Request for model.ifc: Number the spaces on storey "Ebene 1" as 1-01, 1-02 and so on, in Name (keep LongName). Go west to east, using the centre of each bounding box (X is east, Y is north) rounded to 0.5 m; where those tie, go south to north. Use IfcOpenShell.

First a look at what the model holds.

```python
import ifcopenshell
import ifcopenshell.util.element
import ifcopenshell.util.placement

model = ifcopenshell.open("model.ifc")
print(model.schema)
storey = next(s for s in model.by_type("IfcBuildingStorey") if s.Name == "Ebene 1")
spaces = [e for e in ifcopenshell.util.element.get_decomposition(storey) if e.is_a("IfcSpace")]
for e in sorted(spaces, key=lambda e: e.id()):
    origin = ifcopenshell.util.placement.get_local_placement(e.ObjectPlacement)[:3, 3]
    print(e.id(), e.Name, e.LongName, origin.round(2) + 0.0, sep=" | ")
```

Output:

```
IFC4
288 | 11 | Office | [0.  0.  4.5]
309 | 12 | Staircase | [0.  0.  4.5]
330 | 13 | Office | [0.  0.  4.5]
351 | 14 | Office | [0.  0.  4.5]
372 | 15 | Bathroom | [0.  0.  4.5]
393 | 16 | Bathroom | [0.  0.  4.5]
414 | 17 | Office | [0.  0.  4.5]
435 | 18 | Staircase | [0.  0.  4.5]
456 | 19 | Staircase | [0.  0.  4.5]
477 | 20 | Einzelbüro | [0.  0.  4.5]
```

```python
import ifcopenshell
import ifcopenshell.geom
import ifcopenshell.util.element
import ifcopenshell.util.shape

model = ifcopenshell.open("model.ifc")
settings = ifcopenshell.geom.settings()
settings.set("use-world-coords", True)


def centre(element):
    shape = ifcopenshell.geom.create_shape(settings, element)
    return ifcopenshell.util.shape.get_bbox_centroid(shape.geometry)


storey = next(s for s in model.by_type("IfcBuildingStorey") if s.Name == "Ebene 1")
spaces = [e for e in ifcopenshell.util.element.get_decomposition(storey) if e.is_a("IfcSpace")]

# Insertion points can sit at a corner or the storey origin, so sort by the geometry (in metres).
centres = {e: centre(e) for e in spaces}
spaces.sort(key=lambda e: (round(centres[e][0] / 0.5), centres[e][1]))

for i, e in enumerate(spaces, start=1):
    number = f"1-{i:02d}"
    e.Name = number
    print(e.id(), number)

model.write("model_updated.ifc")
```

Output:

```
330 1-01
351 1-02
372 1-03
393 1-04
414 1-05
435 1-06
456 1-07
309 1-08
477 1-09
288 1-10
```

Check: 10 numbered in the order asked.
